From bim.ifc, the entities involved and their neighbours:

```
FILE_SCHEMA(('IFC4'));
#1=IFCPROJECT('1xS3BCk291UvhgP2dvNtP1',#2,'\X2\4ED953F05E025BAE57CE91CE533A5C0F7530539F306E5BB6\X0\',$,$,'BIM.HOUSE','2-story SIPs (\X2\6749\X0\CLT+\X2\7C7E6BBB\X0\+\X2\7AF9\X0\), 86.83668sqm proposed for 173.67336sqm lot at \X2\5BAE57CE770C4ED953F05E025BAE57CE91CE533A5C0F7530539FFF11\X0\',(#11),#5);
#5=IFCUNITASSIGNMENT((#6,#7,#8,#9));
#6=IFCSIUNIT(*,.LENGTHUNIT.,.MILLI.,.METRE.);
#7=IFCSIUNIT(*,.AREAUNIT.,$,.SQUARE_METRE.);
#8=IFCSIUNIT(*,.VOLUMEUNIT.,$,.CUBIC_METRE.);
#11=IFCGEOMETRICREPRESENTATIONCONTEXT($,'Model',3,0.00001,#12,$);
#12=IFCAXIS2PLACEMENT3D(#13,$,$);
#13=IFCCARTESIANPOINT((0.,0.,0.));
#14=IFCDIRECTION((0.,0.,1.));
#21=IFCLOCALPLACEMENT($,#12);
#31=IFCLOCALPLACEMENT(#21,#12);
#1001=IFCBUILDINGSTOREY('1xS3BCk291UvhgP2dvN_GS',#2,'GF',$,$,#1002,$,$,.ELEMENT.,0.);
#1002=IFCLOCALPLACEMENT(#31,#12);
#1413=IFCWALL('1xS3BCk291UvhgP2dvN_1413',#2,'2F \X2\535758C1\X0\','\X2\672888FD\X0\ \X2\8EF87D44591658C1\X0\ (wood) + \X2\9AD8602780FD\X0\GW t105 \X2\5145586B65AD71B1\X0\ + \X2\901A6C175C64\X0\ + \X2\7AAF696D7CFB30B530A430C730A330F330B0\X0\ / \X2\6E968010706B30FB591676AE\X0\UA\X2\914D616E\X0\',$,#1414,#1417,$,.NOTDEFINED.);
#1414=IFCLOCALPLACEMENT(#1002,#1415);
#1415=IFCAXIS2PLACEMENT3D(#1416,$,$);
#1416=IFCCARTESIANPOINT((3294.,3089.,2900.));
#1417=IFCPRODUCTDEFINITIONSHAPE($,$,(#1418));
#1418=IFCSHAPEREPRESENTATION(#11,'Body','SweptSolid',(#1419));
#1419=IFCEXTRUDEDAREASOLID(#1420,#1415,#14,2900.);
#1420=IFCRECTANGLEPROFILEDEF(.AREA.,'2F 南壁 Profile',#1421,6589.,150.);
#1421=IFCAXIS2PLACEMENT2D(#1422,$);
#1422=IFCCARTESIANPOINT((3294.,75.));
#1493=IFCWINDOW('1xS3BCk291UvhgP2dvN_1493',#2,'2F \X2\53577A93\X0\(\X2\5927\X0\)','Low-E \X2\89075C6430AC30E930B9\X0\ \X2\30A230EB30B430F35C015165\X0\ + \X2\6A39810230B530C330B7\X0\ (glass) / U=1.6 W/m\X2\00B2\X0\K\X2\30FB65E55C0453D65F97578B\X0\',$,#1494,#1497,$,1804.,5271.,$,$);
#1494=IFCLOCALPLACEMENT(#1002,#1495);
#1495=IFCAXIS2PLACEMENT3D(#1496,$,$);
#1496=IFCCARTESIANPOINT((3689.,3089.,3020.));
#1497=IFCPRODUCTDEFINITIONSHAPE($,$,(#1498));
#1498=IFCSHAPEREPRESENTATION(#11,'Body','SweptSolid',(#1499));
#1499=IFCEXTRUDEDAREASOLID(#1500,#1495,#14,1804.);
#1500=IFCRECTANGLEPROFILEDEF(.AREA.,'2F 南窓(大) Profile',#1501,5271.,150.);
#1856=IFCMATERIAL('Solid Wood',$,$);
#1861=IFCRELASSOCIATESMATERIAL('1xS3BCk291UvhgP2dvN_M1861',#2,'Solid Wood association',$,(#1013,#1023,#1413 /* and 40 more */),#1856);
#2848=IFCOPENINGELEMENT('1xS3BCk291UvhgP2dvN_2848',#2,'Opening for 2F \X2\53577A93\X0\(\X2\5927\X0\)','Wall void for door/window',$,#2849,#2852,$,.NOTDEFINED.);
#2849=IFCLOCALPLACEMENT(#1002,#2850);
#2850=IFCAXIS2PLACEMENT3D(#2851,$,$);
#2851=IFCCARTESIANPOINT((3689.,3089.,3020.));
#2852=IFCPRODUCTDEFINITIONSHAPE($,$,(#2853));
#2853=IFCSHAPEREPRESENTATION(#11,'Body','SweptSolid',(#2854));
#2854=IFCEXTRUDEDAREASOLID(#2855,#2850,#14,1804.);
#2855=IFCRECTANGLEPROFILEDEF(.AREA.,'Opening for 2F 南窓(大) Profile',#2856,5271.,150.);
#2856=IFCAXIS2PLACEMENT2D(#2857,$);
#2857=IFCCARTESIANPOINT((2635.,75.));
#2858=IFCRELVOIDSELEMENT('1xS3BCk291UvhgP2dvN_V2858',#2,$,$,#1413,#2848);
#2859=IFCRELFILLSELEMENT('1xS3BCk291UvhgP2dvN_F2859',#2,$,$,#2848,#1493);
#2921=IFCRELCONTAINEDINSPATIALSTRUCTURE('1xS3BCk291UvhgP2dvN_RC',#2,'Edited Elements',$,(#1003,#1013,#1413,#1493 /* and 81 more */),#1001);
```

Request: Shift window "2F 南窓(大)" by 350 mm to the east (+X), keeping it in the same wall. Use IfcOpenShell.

```python
import ifcopenshell
import ifcopenshell.api.geometry
import ifcopenshell.util.placement
import ifcopenshell.util.unit

model = ifcopenshell.open("bim.ifc")
unit_scale = ifcopenshell.util.unit.calculate_unit_scale(model)

window = model.by_id(1493)
opening = window.FillsVoids[0].RelatingOpeningElement
wall = opening.VoidsElements[0].RelatingBuildingElement

wall_matrix = ifcopenshell.util.placement.get_local_placement(wall.ObjectPlacement)
shift = wall_matrix[:3, 0] * 0.35 / unit_scale
before = ifcopenshell.util.placement.get_local_placement(window.ObjectPlacement)[:3, 3].copy()

# The window is not placed relative to its opening, so move both.
for product in (opening, window):
    matrix = ifcopenshell.util.placement.get_local_placement(product.ObjectPlacement)
    matrix[:3, 3] += shift
    ifcopenshell.api.geometry.edit_object_placement(model, product=product, matrix=matrix, is_si=False)

after = ifcopenshell.util.placement.get_local_placement(window.ObjectPlacement)[:3, 3]
print("window moved by", (after - before).round(3) + 0.0)

model.write("bim_updated.ifc")
```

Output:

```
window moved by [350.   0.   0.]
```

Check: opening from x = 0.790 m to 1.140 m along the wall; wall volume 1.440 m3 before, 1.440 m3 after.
